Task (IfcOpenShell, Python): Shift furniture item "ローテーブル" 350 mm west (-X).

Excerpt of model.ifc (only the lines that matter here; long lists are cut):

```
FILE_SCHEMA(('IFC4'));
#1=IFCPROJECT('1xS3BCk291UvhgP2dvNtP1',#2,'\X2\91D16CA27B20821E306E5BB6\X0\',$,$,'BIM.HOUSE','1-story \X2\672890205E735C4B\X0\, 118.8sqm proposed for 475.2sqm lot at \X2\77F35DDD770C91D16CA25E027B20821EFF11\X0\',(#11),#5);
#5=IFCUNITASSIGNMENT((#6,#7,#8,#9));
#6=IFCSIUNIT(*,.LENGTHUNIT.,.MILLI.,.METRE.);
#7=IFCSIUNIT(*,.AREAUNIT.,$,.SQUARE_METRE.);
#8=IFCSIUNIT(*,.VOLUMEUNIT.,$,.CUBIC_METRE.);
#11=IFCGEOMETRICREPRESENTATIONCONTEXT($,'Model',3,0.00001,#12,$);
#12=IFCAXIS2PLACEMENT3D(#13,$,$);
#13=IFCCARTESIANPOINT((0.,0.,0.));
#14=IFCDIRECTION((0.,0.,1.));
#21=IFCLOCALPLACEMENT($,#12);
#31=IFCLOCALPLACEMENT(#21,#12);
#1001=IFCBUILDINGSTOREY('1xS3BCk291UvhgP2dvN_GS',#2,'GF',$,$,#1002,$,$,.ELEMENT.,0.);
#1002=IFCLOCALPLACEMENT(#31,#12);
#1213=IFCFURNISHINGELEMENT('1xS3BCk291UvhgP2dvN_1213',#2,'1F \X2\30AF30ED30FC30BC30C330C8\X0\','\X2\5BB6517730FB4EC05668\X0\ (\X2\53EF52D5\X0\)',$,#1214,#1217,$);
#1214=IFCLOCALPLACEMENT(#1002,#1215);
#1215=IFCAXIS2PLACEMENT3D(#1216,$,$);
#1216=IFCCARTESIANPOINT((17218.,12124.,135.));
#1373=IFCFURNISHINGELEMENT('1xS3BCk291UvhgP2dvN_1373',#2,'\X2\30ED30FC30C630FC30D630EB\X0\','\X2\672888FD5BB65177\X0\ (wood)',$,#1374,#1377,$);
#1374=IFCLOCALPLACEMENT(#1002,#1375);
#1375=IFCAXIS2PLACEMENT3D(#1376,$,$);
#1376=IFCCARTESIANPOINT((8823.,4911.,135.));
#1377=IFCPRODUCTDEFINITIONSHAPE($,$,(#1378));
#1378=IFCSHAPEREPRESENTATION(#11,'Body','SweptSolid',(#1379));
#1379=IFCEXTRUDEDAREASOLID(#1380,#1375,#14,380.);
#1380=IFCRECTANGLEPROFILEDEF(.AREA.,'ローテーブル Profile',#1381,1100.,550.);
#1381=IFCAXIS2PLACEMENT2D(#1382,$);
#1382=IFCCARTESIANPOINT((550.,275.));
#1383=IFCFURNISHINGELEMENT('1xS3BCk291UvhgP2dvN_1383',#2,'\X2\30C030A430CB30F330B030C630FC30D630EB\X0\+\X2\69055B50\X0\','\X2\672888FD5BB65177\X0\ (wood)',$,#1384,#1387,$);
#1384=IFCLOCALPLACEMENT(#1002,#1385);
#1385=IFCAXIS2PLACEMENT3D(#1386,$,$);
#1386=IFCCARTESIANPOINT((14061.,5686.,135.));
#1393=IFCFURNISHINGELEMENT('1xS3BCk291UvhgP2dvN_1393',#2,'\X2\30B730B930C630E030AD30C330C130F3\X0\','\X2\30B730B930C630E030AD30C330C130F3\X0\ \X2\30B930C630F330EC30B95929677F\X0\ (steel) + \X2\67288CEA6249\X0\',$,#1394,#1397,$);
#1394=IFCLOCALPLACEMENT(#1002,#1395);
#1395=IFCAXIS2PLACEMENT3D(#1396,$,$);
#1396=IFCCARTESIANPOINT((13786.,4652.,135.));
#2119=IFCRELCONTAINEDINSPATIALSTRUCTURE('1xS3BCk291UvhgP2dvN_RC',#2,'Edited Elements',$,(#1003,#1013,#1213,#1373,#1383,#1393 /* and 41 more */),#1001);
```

```python
import ifcopenshell
import ifcopenshell.api.geometry
import ifcopenshell.util.placement

model = ifcopenshell.open("model.ifc")

item = model.by_id(1373)
matrix = ifcopenshell.util.placement.get_local_placement(item.ObjectPlacement)
matrix[0, 3] -= 350.0
ifcopenshell.api.geometry.edit_object_placement(model, product=item, matrix=matrix, is_si=False)

print(ifcopenshell.util.placement.get_local_placement(item.ObjectPlacement).round(3) + 0.0)

model.write("model_v2.ifc")
```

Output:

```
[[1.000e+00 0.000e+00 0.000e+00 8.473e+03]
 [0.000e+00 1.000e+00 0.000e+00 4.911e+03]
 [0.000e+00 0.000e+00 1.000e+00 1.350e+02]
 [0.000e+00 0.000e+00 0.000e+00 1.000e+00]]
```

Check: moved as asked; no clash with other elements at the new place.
